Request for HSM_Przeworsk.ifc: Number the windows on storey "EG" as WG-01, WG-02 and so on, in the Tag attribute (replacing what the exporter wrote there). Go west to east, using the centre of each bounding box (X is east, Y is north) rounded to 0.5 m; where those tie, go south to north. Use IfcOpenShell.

First a look at what the model holds.

```python
import ifcopenshell
import ifcopenshell.util.element
import ifcopenshell.util.placement

model = ifcopenshell.open("HSM_Przeworsk.ifc")
print(model.schema)
storey = next(s for s in model.by_type("IfcBuildingStorey") if s.Name == "EG")
windows = [e for e in ifcopenshell.util.element.get_decomposition(storey) if e.is_a("IfcWindow")]
for e in sorted(windows, key=lambda e: e.id()):
    origin = ifcopenshell.util.placement.get_local_placement(e.ObjectPlacement)[:3, 3]
    print(e.id(), e.Tag, e.Name, origin.round(2) + 0.0, sep=" | ")
```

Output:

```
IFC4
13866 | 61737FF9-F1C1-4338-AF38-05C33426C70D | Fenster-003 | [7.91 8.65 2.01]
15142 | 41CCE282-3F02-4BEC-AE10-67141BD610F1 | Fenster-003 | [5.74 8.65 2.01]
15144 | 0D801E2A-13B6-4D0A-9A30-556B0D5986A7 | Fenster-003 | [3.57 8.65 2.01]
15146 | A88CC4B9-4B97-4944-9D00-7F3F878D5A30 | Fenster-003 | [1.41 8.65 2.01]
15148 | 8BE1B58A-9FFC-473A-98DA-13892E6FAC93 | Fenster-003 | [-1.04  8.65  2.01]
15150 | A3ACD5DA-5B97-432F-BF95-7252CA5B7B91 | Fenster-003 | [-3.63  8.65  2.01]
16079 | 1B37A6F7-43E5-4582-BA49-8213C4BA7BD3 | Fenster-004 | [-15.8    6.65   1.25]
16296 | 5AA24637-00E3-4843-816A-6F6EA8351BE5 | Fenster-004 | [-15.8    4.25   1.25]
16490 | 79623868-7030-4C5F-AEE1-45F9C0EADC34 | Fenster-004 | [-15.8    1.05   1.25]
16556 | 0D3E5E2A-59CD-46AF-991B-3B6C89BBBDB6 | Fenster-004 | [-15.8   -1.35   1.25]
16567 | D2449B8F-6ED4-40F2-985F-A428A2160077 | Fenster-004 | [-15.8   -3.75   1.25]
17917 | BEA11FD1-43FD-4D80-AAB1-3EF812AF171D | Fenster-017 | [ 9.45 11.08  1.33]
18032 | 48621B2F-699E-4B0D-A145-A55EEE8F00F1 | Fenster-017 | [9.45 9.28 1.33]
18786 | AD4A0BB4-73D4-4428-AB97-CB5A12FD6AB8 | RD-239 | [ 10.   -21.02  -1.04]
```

```python
import ifcopenshell
import ifcopenshell.geom
import ifcopenshell.util.element
import ifcopenshell.util.shape

model = ifcopenshell.open("HSM_Przeworsk.ifc")
settings = ifcopenshell.geom.settings()
settings.set("use-world-coords", True)


def centre(element):
    shape = ifcopenshell.geom.create_shape(settings, element)
    return ifcopenshell.util.shape.get_bbox_centroid(shape.geometry)


storey = next(s for s in model.by_type("IfcBuildingStorey") if s.Name == "EG")
windows = [e for e in ifcopenshell.util.element.get_decomposition(storey) if e.is_a("IfcWindow")]

# Insertion points can sit at a corner or the storey origin, so sort by the geometry (in metres).
centres = {e: centre(e) for e in windows}
windows.sort(key=lambda e: (round(centres[e][0] / 0.5), centres[e][1]))

for i, e in enumerate(windows, start=1):
    number = f"WG-{i:02d}"
    e.Tag = number
    print(e.id(), number)

model.write("HSM_Przeworsk_v2.ifc")
```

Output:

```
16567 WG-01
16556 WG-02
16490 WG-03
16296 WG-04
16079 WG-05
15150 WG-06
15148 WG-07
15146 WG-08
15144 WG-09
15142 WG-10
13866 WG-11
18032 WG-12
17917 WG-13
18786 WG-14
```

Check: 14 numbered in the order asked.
